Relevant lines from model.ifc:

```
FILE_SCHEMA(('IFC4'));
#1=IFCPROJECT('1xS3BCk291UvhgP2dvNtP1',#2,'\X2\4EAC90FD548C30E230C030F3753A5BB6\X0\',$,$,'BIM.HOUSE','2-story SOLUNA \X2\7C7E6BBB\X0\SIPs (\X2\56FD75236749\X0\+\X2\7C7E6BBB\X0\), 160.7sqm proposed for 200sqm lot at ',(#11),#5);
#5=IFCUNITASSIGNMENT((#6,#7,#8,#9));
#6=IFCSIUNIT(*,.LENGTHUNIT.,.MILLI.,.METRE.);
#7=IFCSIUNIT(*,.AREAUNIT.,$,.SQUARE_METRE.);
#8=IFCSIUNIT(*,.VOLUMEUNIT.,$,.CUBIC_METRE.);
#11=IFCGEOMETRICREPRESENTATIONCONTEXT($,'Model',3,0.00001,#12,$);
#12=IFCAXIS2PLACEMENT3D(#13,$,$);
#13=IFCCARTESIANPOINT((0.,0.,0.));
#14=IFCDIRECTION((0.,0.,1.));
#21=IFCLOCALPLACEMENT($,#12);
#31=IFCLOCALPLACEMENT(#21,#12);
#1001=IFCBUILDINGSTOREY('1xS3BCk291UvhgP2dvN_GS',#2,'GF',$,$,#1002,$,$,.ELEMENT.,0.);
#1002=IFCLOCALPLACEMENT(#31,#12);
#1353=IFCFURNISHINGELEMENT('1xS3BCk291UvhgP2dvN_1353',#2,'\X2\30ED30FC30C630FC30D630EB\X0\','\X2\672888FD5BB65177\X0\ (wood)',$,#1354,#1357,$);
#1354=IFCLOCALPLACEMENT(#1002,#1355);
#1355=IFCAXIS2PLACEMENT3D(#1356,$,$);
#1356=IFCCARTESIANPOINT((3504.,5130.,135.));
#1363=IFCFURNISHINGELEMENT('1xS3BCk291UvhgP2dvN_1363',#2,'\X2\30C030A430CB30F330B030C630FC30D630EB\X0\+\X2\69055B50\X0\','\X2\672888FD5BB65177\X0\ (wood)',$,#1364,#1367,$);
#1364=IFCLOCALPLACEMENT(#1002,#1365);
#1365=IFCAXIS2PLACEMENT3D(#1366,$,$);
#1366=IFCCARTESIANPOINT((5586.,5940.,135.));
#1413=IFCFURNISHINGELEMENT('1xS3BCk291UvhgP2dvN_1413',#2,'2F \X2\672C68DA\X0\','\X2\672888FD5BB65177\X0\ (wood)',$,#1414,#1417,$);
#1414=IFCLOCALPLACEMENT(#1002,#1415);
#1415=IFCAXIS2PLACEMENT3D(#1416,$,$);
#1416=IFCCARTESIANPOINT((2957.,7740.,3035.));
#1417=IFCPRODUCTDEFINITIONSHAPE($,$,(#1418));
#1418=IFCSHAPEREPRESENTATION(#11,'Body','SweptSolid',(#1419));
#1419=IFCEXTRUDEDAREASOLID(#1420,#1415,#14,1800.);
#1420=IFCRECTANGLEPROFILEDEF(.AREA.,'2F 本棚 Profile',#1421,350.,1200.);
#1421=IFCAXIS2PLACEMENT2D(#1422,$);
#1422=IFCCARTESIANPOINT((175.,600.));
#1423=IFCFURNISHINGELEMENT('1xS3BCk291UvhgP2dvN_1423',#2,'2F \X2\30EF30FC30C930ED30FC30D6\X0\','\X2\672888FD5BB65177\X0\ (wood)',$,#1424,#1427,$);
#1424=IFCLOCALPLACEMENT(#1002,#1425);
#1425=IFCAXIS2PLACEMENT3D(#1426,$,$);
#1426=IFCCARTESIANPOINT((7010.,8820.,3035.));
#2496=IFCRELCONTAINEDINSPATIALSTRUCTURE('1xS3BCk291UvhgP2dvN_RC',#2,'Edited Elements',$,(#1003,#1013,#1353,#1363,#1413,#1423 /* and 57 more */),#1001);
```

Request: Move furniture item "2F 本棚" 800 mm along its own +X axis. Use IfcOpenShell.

```python
import ifcopenshell
import ifcopenshell.api.geometry
import ifcopenshell.util.placement
import ifcopenshell.util.unit

model = ifcopenshell.open("model.ifc")
unit_scale = ifcopenshell.util.unit.calculate_unit_scale(model)

item = model.by_id(1413)
matrix = ifcopenshell.util.placement.get_local_placement(item.ObjectPlacement)
matrix[:3, 3] += matrix[:3, 0] * 0.8 / unit_scale
ifcopenshell.api.geometry.edit_object_placement(model, product=item, matrix=matrix, is_si=False)

print(ifcopenshell.util.placement.get_local_placement(item.ObjectPlacement).round(3) + 0.0)

model.write("model_rev.ifc")
```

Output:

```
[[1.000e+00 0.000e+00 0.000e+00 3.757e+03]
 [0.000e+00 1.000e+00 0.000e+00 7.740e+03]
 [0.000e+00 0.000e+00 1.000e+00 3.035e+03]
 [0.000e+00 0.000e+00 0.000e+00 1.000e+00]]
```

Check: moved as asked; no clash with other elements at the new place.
